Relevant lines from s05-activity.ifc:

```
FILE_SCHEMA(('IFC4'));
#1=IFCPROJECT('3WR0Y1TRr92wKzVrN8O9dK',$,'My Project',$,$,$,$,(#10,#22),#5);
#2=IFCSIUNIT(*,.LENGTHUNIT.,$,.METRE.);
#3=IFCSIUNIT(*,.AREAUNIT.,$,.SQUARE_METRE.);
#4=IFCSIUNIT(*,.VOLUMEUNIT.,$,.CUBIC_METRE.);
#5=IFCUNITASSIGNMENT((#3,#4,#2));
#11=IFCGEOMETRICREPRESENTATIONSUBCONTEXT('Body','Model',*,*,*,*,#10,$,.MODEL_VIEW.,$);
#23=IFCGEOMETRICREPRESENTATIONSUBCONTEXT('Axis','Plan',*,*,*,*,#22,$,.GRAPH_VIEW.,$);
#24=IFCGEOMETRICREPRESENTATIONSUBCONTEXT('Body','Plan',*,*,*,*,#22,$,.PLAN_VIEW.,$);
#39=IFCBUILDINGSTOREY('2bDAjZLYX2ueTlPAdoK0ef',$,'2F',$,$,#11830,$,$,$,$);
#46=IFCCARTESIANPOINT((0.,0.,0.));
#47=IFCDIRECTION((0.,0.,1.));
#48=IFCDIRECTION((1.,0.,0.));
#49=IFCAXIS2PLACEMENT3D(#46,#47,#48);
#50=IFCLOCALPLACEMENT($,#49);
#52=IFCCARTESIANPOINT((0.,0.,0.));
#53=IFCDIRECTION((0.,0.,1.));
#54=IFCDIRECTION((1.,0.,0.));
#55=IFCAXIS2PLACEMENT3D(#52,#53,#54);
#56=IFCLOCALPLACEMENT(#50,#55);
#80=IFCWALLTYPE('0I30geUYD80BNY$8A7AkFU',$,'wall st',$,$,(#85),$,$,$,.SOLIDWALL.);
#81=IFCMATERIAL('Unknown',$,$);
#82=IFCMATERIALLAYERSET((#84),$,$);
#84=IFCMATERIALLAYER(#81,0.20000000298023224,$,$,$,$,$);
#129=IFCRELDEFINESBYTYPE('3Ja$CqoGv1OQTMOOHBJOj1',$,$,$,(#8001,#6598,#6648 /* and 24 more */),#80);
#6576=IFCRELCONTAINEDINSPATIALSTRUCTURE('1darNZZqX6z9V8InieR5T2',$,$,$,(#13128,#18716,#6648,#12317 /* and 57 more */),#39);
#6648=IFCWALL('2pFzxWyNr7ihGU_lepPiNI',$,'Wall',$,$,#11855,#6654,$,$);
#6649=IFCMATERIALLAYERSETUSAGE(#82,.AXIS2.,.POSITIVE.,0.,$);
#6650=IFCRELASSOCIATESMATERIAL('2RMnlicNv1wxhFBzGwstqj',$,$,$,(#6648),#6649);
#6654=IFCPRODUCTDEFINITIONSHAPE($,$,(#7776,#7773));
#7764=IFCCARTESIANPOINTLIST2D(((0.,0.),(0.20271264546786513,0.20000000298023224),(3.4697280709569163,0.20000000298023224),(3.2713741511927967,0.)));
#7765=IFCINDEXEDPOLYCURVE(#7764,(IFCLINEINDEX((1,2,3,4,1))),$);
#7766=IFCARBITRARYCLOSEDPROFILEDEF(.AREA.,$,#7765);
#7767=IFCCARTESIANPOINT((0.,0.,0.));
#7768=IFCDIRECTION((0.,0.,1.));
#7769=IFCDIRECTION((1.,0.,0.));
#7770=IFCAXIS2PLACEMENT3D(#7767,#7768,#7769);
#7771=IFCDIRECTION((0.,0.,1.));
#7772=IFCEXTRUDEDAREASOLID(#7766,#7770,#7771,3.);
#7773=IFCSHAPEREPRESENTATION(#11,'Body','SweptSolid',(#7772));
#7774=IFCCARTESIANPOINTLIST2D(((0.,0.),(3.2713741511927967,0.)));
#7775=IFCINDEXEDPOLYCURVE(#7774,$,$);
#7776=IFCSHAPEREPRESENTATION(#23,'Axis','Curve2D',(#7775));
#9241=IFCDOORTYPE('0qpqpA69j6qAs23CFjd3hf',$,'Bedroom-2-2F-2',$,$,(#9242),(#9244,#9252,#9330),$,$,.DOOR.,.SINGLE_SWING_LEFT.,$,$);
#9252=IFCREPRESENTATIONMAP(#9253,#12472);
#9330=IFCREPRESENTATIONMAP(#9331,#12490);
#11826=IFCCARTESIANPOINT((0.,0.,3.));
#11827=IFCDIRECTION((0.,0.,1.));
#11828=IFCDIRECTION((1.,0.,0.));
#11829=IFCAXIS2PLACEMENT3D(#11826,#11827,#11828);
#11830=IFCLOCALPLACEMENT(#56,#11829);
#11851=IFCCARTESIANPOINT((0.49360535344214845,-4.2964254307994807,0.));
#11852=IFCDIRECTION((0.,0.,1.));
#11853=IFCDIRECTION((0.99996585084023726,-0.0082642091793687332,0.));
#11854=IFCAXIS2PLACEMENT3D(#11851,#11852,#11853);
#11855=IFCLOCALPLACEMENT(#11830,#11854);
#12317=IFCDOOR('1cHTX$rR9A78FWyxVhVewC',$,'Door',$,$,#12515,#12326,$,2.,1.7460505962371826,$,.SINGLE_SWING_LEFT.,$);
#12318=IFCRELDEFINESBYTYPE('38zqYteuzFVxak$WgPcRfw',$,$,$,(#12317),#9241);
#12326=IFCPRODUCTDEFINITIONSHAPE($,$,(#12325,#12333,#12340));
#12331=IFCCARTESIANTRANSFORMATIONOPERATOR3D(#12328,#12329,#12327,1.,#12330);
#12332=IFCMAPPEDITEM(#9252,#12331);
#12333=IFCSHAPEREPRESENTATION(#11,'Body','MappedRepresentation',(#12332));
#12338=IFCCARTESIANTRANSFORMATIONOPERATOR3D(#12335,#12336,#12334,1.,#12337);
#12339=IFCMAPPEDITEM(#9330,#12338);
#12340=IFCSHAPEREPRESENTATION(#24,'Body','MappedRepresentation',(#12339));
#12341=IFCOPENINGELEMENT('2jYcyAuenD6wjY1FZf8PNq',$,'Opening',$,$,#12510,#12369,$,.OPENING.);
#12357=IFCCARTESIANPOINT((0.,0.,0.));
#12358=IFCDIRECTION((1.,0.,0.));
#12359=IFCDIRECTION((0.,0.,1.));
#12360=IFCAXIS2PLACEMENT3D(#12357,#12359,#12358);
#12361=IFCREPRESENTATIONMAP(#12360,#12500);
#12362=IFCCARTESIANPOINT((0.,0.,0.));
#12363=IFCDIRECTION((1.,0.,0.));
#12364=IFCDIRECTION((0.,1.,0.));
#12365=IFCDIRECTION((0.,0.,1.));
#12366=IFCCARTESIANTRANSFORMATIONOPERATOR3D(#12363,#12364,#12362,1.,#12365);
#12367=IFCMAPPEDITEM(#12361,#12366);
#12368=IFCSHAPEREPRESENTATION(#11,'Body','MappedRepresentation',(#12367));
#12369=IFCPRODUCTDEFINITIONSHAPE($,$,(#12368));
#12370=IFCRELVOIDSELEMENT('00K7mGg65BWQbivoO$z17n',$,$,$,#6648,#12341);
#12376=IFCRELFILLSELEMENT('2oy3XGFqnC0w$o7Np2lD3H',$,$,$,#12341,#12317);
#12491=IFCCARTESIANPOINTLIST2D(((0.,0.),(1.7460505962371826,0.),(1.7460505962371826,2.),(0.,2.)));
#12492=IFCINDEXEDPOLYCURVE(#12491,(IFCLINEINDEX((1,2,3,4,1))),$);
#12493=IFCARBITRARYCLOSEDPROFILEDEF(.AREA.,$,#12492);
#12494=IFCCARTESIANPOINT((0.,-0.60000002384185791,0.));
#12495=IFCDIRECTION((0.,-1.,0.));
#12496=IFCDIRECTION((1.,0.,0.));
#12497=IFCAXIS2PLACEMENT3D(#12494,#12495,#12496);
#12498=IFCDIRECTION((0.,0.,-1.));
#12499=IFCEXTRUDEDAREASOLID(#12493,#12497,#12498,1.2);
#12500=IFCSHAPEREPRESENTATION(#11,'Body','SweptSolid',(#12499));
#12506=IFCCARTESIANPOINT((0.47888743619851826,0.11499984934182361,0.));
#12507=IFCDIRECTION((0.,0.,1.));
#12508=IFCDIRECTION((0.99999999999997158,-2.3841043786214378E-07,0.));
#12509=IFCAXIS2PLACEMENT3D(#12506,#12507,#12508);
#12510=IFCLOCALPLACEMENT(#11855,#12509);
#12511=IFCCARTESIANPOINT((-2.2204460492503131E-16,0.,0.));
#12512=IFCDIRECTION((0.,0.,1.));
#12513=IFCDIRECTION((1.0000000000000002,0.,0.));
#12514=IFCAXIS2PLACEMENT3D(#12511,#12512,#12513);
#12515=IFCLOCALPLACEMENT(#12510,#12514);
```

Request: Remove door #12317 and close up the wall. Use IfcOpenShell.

```python
import ifcopenshell
import ifcopenshell.api.feature
import ifcopenshell.api.root
import ifcopenshell.geom
import ifcopenshell.util.shape

model = ifcopenshell.open("s05-activity.ifc")
settings = ifcopenshell.geom.settings()


def volume(element):
    """Net volume in cubic metres, openings subtracted."""
    shape = ifcopenshell.geom.create_shape(settings, element)
    return ifcopenshell.util.shape.get_volume(shape.geometry)


door = model.by_id(12317)
opening = door.FillsVoids[0].RelatingOpeningElement
wall = opening.VoidsElements[0].RelatingBuildingElement
before = volume(wall)

ifcopenshell.api.root.remove_product(model, product=door)
ifcopenshell.api.feature.remove_feature(model, feature=opening)

after = volume(wall)

print(f"wall volume {before:.3f} -> {after:.3f} m3")

model.write("s05-activity_updated.ifc")
```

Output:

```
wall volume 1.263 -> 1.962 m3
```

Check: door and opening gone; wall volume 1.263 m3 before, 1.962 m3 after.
